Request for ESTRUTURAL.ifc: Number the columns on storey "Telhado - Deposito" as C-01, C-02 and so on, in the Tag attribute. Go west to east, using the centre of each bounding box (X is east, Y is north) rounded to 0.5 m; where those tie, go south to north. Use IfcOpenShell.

First a look at what the model holds.

```python
import ifcopenshell
import ifcopenshell.util.element
import ifcopenshell.util.placement

model = ifcopenshell.open("ESTRUTURAL.ifc")
print(model.schema)
storey = next(s for s in model.by_type("IfcBuildingStorey") if s.Name == "Telhado - Deposito")
columns = [e for e in ifcopenshell.util.element.get_decomposition(storey) if e.is_a("IfcColumn")]
for e in sorted(columns, key=lambda e: e.id()):
    origin = ifcopenshell.util.placement.get_local_placement(e.ObjectPlacement)[:3, 3]
    print(e.id(), e.Tag, e.Name, origin.round(2) + 0.0, sep=" | ")
```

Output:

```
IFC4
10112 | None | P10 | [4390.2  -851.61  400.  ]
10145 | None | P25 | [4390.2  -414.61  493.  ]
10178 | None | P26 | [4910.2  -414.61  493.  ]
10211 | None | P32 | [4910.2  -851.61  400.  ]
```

```python
import ifcopenshell
import ifcopenshell.geom
import ifcopenshell.util.element
import ifcopenshell.util.shape

model = ifcopenshell.open("ESTRUTURAL.ifc")
settings = ifcopenshell.geom.settings()
settings.set("use-world-coords", True)


def centre(element):
    shape = ifcopenshell.geom.create_shape(settings, element)
    return ifcopenshell.util.shape.get_bbox_centroid(shape.geometry)


storey = next(s for s in model.by_type("IfcBuildingStorey") if s.Name == "Telhado - Deposito")
columns = [e for e in ifcopenshell.util.element.get_decomposition(storey) if e.is_a("IfcColumn")]

# Insertion points can sit at a corner or the storey origin, so sort by the geometry (in metres).
centres = {e: centre(e) for e in columns}
columns.sort(key=lambda e: (round(centres[e][0] / 0.5), centres[e][1]))

for i, e in enumerate(columns, start=1):
    number = f"C-{i:02d}"
    e.Tag = number
    print(e.id(), number)

model.write("ESTRUTURAL_updated.ifc")
```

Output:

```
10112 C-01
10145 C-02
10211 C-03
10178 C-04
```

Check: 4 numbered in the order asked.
